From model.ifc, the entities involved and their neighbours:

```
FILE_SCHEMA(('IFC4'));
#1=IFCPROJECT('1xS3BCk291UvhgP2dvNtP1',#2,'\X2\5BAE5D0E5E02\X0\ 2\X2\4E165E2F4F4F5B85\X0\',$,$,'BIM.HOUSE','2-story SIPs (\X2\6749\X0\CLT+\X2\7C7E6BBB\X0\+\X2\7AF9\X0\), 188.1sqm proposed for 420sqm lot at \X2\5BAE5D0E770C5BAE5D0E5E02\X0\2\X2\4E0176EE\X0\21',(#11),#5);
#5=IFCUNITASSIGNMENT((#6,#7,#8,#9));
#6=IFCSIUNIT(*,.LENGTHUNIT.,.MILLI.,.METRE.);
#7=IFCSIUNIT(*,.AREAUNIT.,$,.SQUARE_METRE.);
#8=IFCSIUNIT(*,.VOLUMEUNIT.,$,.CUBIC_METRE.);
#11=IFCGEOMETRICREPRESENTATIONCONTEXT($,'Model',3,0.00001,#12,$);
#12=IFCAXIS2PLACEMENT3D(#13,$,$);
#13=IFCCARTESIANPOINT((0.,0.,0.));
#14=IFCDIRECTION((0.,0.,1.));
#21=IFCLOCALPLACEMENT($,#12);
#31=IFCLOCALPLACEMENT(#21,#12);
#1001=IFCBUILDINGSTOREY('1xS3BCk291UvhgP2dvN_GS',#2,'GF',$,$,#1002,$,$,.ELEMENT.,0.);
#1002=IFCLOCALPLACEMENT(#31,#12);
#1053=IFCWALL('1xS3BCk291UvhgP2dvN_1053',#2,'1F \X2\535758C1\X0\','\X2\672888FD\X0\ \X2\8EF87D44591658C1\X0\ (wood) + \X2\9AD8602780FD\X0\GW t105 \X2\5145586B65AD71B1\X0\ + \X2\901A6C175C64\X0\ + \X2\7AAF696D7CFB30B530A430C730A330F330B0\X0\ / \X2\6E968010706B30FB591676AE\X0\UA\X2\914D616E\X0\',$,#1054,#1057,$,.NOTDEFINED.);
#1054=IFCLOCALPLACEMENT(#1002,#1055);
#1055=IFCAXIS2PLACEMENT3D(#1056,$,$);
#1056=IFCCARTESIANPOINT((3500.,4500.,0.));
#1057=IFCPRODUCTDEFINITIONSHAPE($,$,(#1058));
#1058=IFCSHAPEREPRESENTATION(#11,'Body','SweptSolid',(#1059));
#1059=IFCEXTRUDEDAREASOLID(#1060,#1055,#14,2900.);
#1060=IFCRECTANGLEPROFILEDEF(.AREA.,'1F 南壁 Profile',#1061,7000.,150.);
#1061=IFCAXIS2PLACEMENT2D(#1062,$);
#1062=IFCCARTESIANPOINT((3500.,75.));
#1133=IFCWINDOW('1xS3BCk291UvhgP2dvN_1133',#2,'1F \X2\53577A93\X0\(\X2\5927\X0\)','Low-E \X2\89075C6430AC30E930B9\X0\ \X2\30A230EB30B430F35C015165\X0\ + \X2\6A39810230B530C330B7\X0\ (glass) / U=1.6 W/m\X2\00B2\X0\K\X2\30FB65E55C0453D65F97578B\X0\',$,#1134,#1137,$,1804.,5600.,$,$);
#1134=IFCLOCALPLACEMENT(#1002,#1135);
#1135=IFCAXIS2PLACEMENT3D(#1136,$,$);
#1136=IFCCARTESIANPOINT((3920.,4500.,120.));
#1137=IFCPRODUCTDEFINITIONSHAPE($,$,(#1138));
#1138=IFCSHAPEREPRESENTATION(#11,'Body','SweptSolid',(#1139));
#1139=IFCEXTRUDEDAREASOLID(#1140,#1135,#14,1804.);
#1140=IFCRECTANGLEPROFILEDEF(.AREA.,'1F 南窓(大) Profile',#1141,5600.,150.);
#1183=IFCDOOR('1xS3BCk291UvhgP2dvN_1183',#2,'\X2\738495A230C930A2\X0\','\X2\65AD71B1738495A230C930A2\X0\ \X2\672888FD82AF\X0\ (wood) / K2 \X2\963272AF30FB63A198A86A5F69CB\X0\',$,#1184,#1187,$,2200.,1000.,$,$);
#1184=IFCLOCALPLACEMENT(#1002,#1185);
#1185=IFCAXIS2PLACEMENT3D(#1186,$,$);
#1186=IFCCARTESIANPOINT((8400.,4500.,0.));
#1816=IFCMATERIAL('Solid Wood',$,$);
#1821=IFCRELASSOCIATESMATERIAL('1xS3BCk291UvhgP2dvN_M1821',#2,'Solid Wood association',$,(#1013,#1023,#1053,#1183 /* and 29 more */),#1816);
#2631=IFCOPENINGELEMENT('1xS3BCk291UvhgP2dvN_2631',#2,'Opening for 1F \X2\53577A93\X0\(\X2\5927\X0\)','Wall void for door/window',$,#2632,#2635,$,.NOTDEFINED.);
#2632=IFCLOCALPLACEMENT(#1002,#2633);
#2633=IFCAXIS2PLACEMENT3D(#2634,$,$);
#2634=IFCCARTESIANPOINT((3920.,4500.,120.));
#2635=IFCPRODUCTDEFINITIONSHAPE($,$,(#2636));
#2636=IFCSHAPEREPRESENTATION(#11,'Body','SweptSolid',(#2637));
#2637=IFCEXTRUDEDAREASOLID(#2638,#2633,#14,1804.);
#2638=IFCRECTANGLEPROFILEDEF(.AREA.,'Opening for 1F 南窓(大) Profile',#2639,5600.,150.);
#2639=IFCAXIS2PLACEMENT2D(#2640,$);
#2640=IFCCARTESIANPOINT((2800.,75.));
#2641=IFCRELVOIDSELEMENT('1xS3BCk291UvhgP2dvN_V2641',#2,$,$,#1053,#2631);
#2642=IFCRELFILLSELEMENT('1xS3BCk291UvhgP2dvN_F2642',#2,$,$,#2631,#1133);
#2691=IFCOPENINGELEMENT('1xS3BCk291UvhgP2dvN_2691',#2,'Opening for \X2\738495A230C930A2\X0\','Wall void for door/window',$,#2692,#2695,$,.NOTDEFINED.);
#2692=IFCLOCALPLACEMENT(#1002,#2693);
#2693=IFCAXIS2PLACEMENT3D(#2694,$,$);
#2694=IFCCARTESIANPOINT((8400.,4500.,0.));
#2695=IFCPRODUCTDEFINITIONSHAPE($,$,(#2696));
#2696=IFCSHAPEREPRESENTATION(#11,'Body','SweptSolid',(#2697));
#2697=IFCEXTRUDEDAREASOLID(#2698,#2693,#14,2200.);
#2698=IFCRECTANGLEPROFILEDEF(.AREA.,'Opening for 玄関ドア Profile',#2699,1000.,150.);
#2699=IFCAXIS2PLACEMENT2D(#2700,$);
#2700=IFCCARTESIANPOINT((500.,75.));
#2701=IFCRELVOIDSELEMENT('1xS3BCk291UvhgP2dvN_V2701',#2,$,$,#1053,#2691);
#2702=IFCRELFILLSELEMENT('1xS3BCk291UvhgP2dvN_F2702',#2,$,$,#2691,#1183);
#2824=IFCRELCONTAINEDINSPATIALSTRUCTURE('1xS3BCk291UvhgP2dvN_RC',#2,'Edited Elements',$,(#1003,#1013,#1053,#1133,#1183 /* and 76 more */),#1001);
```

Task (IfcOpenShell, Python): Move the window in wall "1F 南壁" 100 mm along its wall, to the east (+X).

```python
import ifcopenshell
import ifcopenshell.api.geometry
import ifcopenshell.util.placement
import ifcopenshell.util.unit

model = ifcopenshell.open("model.ifc")
unit_scale = ifcopenshell.util.unit.calculate_unit_scale(model)

window = model.by_id(1133)
opening = window.FillsVoids[0].RelatingOpeningElement
wall = opening.VoidsElements[0].RelatingBuildingElement

wall_matrix = ifcopenshell.util.placement.get_local_placement(wall.ObjectPlacement)
shift = wall_matrix[:3, 0] * 0.1 / unit_scale
before = ifcopenshell.util.placement.get_local_placement(window.ObjectPlacement)[:3, 3].copy()

# The window is not placed relative to its opening, so move both.
for product in (opening, window):
    matrix = ifcopenshell.util.placement.get_local_placement(product.ObjectPlacement)
    matrix[:3, 3] += shift
    ifcopenshell.api.geometry.edit_object_placement(model, product=product, matrix=matrix, is_si=False)

after = ifcopenshell.util.placement.get_local_placement(window.ObjectPlacement)[:3, 3]
print("window moved by", (after - before).round(3) + 0.0)

model.write("model_edited.ifc")
```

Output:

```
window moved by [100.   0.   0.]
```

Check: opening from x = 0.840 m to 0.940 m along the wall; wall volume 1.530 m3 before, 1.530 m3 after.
